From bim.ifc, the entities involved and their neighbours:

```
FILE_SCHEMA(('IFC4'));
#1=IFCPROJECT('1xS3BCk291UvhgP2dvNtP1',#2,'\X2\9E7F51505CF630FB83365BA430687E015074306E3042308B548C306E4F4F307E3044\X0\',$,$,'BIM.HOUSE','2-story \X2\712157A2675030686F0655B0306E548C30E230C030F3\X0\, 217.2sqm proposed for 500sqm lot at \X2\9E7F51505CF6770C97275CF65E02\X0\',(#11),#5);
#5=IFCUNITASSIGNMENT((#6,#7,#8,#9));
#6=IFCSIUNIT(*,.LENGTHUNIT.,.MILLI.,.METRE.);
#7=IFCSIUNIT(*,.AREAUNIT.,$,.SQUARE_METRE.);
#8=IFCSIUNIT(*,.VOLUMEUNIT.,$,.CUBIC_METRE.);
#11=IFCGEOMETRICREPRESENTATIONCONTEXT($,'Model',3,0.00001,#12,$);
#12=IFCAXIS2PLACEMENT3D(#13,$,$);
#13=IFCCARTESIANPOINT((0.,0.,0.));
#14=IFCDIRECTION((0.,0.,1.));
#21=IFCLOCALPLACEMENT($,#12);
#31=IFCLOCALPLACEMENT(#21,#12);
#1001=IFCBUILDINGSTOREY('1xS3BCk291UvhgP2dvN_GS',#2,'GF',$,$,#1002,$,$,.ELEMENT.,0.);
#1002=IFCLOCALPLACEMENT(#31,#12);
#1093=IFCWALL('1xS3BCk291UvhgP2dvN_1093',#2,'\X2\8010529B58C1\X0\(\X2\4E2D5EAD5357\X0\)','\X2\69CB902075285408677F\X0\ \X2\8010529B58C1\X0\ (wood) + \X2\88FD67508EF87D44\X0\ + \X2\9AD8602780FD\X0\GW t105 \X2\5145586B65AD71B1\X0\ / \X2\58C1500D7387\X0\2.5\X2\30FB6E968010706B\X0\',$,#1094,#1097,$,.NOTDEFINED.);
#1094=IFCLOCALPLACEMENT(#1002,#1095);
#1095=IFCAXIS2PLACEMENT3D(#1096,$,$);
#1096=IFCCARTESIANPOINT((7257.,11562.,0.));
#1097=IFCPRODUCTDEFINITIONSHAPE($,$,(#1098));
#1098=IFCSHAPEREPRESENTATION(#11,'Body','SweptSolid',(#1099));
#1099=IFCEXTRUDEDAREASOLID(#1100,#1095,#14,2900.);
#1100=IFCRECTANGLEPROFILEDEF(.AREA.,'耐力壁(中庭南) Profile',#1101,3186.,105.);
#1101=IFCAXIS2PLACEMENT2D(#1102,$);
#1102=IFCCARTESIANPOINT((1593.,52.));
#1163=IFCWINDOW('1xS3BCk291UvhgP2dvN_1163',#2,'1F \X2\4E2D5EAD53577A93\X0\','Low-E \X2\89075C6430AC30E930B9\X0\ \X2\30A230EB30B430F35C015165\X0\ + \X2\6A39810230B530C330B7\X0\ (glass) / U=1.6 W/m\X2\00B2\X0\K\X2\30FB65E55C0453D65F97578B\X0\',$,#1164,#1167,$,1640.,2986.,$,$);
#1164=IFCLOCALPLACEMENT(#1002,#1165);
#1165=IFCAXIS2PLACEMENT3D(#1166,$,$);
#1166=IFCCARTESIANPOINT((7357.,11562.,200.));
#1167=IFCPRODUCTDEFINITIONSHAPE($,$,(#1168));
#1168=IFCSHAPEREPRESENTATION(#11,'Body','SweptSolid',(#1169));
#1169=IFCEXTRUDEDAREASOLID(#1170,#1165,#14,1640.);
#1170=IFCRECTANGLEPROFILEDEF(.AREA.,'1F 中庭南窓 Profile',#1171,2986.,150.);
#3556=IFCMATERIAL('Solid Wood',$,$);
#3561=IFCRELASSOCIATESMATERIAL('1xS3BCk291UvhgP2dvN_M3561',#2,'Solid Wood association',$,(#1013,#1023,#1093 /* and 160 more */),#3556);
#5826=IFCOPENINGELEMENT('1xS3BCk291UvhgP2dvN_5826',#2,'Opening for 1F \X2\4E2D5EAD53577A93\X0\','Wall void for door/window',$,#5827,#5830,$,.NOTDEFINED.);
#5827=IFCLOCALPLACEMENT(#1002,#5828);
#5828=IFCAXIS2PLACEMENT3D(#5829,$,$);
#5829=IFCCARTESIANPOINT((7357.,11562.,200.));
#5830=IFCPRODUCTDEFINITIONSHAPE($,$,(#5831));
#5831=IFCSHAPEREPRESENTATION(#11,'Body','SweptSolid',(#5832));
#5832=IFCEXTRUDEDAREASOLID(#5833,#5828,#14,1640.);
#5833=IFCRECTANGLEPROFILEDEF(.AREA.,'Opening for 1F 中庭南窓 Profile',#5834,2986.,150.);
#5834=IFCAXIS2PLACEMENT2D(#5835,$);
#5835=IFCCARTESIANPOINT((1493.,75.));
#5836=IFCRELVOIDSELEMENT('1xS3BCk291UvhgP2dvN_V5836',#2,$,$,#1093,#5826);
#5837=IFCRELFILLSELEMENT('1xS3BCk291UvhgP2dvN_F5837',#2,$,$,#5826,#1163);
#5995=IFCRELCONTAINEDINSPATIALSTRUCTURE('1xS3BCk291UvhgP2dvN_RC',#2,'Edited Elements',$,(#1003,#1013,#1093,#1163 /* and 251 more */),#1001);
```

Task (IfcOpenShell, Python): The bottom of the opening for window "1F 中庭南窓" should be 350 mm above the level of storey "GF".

```python
import numpy as np
import ifcopenshell
import ifcopenshell.api.geometry
import ifcopenshell.geom
import ifcopenshell.util.element
import ifcopenshell.util.placement
import ifcopenshell.util.shape
import ifcopenshell.util.unit

model = ifcopenshell.open("bim.ifc")
unit_scale = ifcopenshell.util.unit.calculate_unit_scale(model)

window = model.by_id(1163)
opening = window.FillsVoids[0].RelatingOpeningElement
storey = ifcopenshell.util.element.get_container(window, ifc_class="IfcBuildingStorey")
level = ifcopenshell.util.placement.get_local_placement(storey.ObjectPlacement)[2, 3]

# The opening's origin need not be at the sill, so measure its lowest point.
shape = ifcopenshell.geom.create_shape(ifcopenshell.geom.settings(), opening)
bottom = ifcopenshell.util.shape.get_shape_bottom_elevation(shape, shape.geometry) / unit_scale
dz = level + 350.0 - bottom

shift = np.array([0.0, 0.0, dz])
# The window is not placed relative to its opening, so move both.
for product in (opening, window):
    matrix = ifcopenshell.util.placement.get_local_placement(product.ObjectPlacement)
    matrix[:3, 3] += shift
    ifcopenshell.api.geometry.edit_object_placement(model, product=product, matrix=matrix, is_si=False)

print(f"moved by {dz * unit_scale:+.3f} m")

model.write("bim_rev.ifc")
```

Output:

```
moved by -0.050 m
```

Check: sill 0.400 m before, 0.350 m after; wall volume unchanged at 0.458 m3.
